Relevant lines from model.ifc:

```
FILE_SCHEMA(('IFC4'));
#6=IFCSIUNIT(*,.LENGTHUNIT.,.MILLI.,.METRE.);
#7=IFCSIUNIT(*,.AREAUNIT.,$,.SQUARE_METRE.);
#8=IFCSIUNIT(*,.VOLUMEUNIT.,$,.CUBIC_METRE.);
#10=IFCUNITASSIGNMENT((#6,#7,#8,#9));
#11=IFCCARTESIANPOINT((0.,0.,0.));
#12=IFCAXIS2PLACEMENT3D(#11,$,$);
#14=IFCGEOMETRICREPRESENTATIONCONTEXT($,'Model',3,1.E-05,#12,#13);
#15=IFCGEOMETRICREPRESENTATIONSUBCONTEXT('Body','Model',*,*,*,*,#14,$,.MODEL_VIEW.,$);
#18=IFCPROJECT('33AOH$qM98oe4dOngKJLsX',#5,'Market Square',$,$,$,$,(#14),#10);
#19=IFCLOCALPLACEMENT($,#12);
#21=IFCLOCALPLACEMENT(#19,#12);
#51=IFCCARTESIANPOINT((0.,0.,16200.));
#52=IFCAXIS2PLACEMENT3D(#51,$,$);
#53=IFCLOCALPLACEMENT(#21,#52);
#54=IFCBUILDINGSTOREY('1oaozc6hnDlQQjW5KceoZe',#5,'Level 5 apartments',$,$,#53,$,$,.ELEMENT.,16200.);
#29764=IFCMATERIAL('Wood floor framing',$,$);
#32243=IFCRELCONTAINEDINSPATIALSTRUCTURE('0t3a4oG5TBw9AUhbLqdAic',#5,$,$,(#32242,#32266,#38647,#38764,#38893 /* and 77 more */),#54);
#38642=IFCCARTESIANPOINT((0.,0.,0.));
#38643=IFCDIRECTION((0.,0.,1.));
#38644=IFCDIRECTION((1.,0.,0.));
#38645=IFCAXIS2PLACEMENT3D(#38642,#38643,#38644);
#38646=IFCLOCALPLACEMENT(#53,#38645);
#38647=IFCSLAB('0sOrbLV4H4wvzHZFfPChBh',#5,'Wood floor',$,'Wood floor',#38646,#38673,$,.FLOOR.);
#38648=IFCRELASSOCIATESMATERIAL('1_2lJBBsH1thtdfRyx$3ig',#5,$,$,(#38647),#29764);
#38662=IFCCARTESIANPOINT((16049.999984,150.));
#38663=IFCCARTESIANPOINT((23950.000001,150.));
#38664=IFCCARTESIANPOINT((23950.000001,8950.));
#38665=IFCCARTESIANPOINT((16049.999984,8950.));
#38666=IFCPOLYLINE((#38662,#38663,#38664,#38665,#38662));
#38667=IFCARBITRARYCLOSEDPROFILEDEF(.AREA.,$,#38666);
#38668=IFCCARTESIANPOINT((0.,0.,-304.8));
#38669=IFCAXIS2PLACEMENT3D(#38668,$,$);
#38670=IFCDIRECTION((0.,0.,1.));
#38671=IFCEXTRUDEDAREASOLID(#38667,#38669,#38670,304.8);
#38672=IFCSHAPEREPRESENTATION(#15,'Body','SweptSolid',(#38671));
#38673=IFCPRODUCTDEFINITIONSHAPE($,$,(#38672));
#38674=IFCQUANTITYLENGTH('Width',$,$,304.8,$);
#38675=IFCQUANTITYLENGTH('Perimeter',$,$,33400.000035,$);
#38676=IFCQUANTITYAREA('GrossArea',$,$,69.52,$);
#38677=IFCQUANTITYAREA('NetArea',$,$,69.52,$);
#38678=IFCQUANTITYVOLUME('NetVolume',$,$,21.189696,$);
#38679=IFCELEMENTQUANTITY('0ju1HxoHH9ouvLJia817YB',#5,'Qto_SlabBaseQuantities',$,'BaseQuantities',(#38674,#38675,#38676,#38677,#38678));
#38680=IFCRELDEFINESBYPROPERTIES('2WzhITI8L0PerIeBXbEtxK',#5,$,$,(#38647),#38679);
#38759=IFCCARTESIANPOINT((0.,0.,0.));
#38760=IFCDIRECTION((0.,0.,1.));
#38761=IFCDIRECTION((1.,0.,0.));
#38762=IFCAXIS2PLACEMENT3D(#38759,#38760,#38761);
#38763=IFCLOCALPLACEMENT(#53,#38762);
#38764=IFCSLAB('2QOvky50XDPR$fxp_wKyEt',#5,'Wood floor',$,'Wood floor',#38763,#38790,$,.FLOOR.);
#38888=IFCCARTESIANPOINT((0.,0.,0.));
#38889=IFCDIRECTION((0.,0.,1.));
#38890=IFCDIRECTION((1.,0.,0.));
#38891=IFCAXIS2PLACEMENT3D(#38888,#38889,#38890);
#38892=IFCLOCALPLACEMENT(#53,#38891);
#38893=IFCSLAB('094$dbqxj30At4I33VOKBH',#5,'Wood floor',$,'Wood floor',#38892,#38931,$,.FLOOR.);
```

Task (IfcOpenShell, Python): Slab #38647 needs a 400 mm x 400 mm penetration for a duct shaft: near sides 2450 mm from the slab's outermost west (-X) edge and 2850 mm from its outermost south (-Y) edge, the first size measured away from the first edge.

```python
import numpy as np
import ifcopenshell
import ifcopenshell.api.feature
import ifcopenshell.api.geometry
import ifcopenshell.api.pset
import ifcopenshell.api.root
import ifcopenshell.geom
import ifcopenshell.util.element
import ifcopenshell.util.placement
import ifcopenshell.util.representation
import ifcopenshell.util.shape
import ifcopenshell.util.unit

model = ifcopenshell.open("model.ifc")
unit_scale = ifcopenshell.util.unit.calculate_unit_scale(model)
area_scale = ifcopenshell.util.unit.calculate_unit_scale(model, "AREAUNIT")
volume_scale = ifcopenshell.util.unit.calculate_unit_scale(model, "VOLUMEUNIT")
settings = ifcopenshell.geom.settings()


def volume(element):
    """Net volume in cubic metres, openings subtracted."""
    shape = ifcopenshell.geom.create_shape(settings, element)
    return ifcopenshell.util.shape.get_volume(shape.geometry)


slab = model.by_id(38647)
before = volume(slab)

# Extent in the slab's own axes, in metres. The edges named are its -X and -Y sides.
slab_shape = ifcopenshell.geom.create_shape(settings, slab)
vertices = ifcopenshell.util.shape.get_vertices(slab_shape.geometry)
x_min, y_min, bottom = vertices.min(axis=0)
top = vertices[:, 2].max()

opening = ifcopenshell.api.root.create_entity(model, ifc_class="IfcOpeningElement", name="Duct shaft opening", predefined_type="OPENING")
context = ifcopenshell.util.representation.get_context(model, "Model", "Body", "MODEL_VIEW")
width, depth = 0.4, 0.4
outline = [(0.0, 0.0), (width, 0.0), (width, depth), (0.0, depth), (0.0, 0.0)]
# Overshoot both faces by 50 mm so the cut is clean.
shape = ifcopenshell.api.geometry.add_slab_representation(
    model, context=context, depth=top - bottom + 0.1, polyline=outline
)
ifcopenshell.api.geometry.assign_representation(model, product=opening, representation=shape)

matrix = ifcopenshell.util.placement.get_local_placement(slab.ObjectPlacement)
matrix[:, 3] = matrix @ np.append(np.array([x_min + 2.45, y_min + 2.85, bottom - 0.05]) / unit_scale, 1.0)
ifcopenshell.api.geometry.edit_object_placement(model, product=opening, matrix=matrix, is_si=False)
ifcopenshell.api.feature.add_feature(model, feature=opening, element=slab)

after = volume(slab)

# Update the slab's stored quantities.
qto = model.by_id(ifcopenshell.util.element.get_pset(slab, "Qto_SlabBaseQuantities", should_inherit=False)["id"])
ifcopenshell.api.pset.edit_qto(model, qto=qto, properties={
    "NetArea": after / (top - bottom) / area_scale,
    "NetVolume": after / volume_scale,
})

print(f"slab volume {before:.3f} -> {after:.3f} m3")

model.write("model_updated.ifc")
```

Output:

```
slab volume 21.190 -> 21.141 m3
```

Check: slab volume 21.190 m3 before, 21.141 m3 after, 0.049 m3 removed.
